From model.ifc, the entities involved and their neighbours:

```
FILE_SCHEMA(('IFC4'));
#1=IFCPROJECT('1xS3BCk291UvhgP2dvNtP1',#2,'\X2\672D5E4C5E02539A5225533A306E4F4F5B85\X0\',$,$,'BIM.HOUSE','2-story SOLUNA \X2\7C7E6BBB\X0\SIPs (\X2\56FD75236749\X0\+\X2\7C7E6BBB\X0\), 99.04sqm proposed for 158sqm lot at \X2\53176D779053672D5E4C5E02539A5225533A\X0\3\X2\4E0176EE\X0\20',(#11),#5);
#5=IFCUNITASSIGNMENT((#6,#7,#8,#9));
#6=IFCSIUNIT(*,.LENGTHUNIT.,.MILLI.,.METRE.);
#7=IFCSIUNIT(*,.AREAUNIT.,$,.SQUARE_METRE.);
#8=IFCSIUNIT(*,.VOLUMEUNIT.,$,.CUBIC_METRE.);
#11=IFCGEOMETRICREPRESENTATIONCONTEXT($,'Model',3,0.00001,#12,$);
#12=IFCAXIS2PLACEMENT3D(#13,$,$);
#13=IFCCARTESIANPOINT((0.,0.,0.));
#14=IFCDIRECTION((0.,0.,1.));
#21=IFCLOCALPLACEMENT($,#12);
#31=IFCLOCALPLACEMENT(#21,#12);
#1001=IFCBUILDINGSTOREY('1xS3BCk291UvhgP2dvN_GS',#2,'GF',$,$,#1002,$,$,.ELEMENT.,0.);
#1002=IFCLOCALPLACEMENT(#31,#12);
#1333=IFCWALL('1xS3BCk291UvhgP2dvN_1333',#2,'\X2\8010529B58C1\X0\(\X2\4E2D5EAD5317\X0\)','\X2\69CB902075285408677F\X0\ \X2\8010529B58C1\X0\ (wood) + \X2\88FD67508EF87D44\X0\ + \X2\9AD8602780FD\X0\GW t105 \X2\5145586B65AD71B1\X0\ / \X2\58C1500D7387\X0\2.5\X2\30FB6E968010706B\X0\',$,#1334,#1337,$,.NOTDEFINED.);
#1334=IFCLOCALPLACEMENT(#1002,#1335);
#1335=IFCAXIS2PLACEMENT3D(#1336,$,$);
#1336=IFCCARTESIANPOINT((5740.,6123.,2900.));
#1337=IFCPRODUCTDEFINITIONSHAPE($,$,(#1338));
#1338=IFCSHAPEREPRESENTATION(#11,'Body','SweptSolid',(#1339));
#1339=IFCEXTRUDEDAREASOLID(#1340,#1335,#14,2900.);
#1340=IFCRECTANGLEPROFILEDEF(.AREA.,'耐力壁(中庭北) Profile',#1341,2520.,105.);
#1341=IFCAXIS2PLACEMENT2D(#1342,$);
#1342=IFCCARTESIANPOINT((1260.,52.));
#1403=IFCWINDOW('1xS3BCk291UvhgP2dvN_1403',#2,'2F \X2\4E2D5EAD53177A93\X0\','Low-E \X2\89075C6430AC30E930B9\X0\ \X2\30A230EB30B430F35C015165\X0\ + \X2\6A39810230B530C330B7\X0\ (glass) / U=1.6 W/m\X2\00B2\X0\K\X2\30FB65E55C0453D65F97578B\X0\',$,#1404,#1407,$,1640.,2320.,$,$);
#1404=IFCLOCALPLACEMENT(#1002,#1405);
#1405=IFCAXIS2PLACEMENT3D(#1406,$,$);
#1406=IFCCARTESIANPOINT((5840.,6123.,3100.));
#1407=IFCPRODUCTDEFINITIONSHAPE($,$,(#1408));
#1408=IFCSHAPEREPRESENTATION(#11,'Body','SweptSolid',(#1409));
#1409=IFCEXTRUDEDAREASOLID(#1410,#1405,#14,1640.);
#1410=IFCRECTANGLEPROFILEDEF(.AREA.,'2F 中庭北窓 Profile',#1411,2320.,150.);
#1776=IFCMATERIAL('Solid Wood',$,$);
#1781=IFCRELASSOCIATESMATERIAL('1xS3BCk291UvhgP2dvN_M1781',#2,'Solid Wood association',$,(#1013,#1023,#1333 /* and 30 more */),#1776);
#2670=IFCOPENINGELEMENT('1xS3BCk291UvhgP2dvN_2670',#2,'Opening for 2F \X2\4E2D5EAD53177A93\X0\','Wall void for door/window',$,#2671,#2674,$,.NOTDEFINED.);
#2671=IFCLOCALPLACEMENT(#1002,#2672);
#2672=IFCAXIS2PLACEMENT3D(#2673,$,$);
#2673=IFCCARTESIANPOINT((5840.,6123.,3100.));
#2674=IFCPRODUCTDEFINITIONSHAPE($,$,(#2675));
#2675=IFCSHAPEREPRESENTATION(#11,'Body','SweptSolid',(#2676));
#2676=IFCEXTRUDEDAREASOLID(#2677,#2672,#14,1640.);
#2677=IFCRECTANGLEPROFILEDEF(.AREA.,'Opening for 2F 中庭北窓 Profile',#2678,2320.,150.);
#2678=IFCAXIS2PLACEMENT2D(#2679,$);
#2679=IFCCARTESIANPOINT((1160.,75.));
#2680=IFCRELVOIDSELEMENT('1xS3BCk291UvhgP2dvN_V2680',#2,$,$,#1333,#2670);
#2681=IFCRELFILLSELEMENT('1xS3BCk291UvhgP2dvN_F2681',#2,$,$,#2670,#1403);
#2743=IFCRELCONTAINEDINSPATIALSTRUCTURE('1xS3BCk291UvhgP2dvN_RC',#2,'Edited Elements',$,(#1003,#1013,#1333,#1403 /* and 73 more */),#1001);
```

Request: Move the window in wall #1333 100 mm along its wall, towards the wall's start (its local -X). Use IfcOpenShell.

```python
import ifcopenshell
import ifcopenshell.api.geometry
import ifcopenshell.util.placement

model = ifcopenshell.open("model.ifc")

window = model.by_guid("1xS3BCk291UvhgP2dvN_1403")
opening = window.FillsVoids[0].RelatingOpeningElement
wall = opening.VoidsElements[0].RelatingBuildingElement

wall_matrix = ifcopenshell.util.placement.get_local_placement(wall.ObjectPlacement)
shift = wall_matrix[:3, 0] * -100.0
before = ifcopenshell.util.placement.get_local_placement(window.ObjectPlacement)[:3, 3].copy()

# The window is not placed relative to its opening, so move both.
for product in (opening, window):
    matrix = ifcopenshell.util.placement.get_local_placement(product.ObjectPlacement)
    matrix[:3, 3] += shift
    ifcopenshell.api.geometry.edit_object_placement(model, product=product, matrix=matrix, is_si=False)

after = ifcopenshell.util.placement.get_local_placement(window.ObjectPlacement)[:3, 3]
print("window moved by", (after - before).round(3) + 0.0)

model.write("model-out.ifc")
```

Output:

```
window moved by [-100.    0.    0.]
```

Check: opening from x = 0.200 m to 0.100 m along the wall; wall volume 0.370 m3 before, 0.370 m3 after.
